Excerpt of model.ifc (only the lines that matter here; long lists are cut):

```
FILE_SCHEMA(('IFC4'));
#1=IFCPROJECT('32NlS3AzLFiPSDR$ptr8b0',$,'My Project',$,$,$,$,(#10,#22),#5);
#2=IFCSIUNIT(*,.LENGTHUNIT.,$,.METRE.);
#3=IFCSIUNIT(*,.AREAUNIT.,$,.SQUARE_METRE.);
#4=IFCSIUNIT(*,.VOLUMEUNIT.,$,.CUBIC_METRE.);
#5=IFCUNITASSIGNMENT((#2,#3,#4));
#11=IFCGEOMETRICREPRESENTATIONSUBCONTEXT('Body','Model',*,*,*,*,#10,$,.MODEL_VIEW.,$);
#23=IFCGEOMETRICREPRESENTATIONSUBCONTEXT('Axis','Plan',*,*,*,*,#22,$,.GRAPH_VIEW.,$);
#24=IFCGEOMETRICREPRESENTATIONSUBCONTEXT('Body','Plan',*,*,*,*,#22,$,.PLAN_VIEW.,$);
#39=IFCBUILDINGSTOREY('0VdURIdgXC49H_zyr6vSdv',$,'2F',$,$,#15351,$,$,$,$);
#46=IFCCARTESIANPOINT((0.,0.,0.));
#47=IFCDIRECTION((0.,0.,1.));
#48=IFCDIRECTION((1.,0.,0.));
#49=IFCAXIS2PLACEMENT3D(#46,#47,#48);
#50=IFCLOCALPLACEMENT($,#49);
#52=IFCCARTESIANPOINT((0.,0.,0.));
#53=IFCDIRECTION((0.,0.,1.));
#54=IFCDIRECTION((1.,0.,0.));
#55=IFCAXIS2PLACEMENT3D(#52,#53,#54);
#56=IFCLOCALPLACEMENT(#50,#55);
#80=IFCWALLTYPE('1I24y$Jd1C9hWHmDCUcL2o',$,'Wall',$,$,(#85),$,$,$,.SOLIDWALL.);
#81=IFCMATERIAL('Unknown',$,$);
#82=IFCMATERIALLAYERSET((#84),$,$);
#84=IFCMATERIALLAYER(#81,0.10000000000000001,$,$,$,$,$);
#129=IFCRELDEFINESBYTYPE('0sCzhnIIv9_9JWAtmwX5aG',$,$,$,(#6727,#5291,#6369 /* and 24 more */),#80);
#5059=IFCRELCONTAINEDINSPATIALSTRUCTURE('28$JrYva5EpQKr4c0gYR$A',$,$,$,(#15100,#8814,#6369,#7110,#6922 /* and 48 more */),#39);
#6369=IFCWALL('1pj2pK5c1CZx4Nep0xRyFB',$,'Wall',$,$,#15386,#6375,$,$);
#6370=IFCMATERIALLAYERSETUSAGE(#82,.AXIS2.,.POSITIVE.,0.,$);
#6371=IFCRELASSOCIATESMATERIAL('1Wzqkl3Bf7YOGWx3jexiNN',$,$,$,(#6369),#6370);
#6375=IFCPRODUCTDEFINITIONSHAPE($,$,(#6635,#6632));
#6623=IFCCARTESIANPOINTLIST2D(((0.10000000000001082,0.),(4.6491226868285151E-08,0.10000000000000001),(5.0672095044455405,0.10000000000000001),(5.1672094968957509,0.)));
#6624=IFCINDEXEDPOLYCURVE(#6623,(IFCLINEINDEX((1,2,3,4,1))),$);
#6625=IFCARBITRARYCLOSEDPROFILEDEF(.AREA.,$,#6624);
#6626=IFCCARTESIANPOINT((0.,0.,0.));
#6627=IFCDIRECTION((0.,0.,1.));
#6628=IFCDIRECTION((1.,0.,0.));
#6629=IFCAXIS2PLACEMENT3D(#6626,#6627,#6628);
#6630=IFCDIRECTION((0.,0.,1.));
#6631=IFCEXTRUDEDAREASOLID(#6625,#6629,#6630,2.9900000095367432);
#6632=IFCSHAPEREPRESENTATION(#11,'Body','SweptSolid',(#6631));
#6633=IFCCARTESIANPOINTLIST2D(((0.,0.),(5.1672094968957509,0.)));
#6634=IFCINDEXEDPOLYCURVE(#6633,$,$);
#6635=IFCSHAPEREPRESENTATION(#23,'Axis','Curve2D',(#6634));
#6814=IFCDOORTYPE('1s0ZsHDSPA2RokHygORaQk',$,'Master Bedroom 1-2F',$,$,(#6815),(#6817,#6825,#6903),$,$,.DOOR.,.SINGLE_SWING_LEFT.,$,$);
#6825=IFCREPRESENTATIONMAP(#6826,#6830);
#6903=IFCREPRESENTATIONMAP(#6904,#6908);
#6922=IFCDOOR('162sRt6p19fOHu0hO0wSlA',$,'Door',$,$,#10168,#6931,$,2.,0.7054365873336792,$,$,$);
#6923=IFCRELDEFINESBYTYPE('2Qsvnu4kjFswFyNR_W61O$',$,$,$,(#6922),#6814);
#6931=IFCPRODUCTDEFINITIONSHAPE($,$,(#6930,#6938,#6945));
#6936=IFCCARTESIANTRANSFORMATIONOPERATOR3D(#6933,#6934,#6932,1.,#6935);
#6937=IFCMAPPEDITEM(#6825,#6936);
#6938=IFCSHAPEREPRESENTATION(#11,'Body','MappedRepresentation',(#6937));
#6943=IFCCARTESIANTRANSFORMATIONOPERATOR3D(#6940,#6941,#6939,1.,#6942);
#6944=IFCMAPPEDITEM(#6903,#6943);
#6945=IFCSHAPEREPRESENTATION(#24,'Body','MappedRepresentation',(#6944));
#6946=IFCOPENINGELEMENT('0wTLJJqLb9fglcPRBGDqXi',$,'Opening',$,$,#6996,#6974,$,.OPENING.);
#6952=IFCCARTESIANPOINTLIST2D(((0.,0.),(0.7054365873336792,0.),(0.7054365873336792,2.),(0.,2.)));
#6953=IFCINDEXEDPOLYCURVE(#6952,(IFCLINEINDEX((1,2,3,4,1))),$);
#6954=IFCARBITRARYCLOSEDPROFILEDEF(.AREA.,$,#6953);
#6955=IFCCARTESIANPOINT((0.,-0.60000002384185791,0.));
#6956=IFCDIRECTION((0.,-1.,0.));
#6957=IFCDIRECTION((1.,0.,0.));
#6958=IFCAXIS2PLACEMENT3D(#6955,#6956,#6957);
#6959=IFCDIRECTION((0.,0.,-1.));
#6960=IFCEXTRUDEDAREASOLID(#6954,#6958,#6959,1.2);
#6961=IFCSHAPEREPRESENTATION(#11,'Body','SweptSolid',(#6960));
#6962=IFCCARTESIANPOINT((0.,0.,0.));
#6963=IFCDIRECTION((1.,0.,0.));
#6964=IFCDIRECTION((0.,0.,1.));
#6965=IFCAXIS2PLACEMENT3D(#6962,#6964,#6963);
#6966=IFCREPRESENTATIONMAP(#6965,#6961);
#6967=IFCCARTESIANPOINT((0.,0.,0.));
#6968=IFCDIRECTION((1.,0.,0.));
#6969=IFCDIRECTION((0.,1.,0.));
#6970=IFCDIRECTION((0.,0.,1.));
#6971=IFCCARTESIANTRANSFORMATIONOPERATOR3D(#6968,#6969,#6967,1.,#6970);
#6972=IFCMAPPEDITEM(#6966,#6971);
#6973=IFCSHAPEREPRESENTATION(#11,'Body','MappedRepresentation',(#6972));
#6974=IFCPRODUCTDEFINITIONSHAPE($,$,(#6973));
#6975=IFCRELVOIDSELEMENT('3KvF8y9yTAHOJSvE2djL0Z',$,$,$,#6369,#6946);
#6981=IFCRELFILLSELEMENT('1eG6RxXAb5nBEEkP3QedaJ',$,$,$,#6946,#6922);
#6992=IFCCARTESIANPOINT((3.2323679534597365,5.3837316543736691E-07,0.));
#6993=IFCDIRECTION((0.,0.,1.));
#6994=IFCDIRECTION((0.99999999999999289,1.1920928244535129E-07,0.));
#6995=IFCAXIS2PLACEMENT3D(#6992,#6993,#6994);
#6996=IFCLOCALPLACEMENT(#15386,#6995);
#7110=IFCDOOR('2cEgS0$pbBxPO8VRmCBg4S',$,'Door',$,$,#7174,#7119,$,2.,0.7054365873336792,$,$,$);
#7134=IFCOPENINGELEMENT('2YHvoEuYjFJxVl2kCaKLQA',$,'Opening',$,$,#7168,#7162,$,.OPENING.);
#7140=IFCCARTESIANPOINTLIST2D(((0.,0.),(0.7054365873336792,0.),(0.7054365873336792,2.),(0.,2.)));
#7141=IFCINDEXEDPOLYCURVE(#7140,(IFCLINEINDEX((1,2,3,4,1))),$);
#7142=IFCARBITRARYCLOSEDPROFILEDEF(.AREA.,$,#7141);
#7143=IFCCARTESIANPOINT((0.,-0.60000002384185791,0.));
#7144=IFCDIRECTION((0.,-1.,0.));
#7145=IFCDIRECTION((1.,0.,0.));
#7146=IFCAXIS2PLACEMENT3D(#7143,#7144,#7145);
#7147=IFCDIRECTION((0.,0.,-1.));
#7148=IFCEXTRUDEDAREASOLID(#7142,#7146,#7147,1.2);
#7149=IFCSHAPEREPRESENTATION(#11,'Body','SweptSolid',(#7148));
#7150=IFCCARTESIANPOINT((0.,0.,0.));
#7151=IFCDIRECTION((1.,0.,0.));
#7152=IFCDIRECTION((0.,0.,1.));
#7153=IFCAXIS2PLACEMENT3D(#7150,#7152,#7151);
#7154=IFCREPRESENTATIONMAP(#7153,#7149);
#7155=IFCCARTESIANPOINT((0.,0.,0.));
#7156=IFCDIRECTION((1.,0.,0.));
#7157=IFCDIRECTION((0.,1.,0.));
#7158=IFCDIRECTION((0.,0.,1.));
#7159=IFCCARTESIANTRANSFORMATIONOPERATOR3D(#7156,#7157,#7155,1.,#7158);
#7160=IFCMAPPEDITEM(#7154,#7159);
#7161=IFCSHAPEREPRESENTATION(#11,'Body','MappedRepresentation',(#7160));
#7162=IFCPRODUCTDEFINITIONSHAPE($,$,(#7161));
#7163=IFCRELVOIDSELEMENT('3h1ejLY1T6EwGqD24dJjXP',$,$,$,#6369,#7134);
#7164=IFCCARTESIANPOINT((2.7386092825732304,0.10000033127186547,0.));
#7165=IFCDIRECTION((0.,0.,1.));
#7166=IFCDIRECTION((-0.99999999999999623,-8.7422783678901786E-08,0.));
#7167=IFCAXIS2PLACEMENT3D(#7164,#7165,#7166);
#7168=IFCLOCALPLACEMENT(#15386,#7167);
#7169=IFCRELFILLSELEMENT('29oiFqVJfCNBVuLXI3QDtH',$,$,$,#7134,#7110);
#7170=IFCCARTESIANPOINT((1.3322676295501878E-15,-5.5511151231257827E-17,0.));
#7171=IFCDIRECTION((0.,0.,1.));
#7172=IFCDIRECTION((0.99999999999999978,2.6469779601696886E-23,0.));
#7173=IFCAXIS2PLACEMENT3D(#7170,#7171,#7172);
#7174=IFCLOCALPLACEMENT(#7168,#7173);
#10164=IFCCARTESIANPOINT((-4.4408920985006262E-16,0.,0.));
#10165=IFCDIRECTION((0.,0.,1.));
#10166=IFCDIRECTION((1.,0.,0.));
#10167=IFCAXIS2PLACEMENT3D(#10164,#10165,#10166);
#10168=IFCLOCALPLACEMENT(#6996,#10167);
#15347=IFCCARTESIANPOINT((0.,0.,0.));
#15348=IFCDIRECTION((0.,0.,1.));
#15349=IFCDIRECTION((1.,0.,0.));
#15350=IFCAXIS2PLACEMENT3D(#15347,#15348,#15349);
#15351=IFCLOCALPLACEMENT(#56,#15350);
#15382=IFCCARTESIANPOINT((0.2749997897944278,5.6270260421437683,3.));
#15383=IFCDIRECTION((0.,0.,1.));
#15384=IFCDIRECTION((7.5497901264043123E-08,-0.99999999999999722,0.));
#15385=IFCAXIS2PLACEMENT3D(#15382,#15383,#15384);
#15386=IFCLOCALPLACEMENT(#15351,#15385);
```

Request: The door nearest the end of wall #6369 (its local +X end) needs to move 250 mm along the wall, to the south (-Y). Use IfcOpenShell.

```python
import ifcopenshell
import ifcopenshell.api.geometry
import ifcopenshell.util.placement
import ifcopenshell.util.unit

model = ifcopenshell.open("model.ifc")
unit_scale = ifcopenshell.util.unit.calculate_unit_scale(model)

door = model.by_guid("162sRt6p19fOHu0hO0wSlA")
opening = door.FillsVoids[0].RelatingOpeningElement
wall = opening.VoidsElements[0].RelatingBuildingElement

wall_matrix = ifcopenshell.util.placement.get_local_placement(wall.ObjectPlacement)
shift = wall_matrix[:3, 0] * 0.25 / unit_scale
before = ifcopenshell.util.placement.get_local_placement(door.ObjectPlacement)[:3, 3].copy()

# The door is placed relative to its opening, so it follows when the opening moves.
matrix = ifcopenshell.util.placement.get_local_placement(opening.ObjectPlacement)
matrix[:3, 3] += shift
ifcopenshell.api.geometry.edit_object_placement(
    model, product=opening, matrix=matrix, is_si=False, should_transform_children=True
)

after = ifcopenshell.util.placement.get_local_placement(door.ObjectPlacement)[:3, 3]
print("door moved by", (after - before).round(3) + 0.0)

model.write("model-out.ifc")
```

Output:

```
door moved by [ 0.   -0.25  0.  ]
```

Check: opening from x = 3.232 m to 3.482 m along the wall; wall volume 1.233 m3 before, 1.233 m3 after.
